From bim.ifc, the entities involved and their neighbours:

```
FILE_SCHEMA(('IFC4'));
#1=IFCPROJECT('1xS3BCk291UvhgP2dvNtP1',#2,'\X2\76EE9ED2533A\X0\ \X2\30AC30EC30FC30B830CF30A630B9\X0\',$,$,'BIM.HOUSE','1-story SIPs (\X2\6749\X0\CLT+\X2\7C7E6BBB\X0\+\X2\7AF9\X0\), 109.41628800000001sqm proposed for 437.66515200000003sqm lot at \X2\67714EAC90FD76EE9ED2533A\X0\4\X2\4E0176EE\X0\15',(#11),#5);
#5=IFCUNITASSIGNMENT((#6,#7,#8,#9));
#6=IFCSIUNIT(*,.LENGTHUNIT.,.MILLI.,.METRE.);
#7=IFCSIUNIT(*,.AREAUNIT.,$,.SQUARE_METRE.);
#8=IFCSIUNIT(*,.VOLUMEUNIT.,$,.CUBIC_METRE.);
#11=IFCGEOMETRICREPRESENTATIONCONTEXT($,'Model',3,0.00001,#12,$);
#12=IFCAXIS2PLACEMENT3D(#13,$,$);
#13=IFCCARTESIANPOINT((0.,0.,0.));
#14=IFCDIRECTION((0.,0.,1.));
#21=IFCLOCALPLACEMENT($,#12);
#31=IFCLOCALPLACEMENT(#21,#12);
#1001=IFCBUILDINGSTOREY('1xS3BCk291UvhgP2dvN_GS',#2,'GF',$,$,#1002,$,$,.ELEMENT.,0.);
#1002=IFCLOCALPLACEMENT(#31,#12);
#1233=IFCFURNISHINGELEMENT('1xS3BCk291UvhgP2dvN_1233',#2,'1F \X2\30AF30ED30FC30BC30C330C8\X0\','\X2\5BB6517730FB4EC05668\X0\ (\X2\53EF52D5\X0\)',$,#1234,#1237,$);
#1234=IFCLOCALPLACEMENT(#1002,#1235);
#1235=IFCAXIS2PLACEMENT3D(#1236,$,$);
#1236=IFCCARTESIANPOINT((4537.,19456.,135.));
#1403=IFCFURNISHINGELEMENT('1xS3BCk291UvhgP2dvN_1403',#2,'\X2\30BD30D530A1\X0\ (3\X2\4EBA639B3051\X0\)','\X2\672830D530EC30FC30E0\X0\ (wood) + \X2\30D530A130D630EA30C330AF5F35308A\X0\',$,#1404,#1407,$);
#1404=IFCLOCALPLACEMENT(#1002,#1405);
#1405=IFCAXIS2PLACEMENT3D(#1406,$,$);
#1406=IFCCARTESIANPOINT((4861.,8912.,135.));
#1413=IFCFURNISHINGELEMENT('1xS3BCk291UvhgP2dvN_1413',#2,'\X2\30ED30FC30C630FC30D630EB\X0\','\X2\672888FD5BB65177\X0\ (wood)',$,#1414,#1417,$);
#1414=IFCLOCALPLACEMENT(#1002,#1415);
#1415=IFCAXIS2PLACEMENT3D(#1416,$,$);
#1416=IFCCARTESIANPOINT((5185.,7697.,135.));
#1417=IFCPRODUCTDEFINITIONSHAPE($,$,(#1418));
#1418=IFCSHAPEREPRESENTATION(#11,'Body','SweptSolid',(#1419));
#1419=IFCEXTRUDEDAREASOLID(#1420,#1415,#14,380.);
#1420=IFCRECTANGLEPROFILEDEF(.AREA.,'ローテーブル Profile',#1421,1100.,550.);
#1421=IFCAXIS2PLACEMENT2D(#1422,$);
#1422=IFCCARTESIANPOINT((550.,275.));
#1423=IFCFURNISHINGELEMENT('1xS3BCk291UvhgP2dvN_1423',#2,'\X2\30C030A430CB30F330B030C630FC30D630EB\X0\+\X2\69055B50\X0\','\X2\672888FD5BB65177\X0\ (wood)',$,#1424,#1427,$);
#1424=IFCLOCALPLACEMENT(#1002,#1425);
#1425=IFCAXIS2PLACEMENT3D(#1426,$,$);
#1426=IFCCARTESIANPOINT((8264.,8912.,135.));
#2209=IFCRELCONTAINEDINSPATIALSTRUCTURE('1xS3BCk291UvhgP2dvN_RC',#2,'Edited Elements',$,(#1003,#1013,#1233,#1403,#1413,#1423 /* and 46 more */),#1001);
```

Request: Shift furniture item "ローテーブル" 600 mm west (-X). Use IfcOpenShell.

```python
import ifcopenshell
import ifcopenshell.api.geometry
import ifcopenshell.util.placement
import ifcopenshell.util.unit

model = ifcopenshell.open("bim.ifc")
unit_scale = ifcopenshell.util.unit.calculate_unit_scale(model)

item = model.by_guid("1xS3BCk291UvhgP2dvN_1413")
matrix = ifcopenshell.util.placement.get_local_placement(item.ObjectPlacement)
matrix[0, 3] -= 0.6 / unit_scale
ifcopenshell.api.geometry.edit_object_placement(model, product=item, matrix=matrix, is_si=False)

print(ifcopenshell.util.placement.get_local_placement(item.ObjectPlacement).round(3) + 0.0)

model.write("bim_edited.ifc")
```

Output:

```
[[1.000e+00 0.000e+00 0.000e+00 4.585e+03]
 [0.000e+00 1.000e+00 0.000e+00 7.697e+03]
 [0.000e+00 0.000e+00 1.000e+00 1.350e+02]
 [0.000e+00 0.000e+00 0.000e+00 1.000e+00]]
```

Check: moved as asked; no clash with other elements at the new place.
